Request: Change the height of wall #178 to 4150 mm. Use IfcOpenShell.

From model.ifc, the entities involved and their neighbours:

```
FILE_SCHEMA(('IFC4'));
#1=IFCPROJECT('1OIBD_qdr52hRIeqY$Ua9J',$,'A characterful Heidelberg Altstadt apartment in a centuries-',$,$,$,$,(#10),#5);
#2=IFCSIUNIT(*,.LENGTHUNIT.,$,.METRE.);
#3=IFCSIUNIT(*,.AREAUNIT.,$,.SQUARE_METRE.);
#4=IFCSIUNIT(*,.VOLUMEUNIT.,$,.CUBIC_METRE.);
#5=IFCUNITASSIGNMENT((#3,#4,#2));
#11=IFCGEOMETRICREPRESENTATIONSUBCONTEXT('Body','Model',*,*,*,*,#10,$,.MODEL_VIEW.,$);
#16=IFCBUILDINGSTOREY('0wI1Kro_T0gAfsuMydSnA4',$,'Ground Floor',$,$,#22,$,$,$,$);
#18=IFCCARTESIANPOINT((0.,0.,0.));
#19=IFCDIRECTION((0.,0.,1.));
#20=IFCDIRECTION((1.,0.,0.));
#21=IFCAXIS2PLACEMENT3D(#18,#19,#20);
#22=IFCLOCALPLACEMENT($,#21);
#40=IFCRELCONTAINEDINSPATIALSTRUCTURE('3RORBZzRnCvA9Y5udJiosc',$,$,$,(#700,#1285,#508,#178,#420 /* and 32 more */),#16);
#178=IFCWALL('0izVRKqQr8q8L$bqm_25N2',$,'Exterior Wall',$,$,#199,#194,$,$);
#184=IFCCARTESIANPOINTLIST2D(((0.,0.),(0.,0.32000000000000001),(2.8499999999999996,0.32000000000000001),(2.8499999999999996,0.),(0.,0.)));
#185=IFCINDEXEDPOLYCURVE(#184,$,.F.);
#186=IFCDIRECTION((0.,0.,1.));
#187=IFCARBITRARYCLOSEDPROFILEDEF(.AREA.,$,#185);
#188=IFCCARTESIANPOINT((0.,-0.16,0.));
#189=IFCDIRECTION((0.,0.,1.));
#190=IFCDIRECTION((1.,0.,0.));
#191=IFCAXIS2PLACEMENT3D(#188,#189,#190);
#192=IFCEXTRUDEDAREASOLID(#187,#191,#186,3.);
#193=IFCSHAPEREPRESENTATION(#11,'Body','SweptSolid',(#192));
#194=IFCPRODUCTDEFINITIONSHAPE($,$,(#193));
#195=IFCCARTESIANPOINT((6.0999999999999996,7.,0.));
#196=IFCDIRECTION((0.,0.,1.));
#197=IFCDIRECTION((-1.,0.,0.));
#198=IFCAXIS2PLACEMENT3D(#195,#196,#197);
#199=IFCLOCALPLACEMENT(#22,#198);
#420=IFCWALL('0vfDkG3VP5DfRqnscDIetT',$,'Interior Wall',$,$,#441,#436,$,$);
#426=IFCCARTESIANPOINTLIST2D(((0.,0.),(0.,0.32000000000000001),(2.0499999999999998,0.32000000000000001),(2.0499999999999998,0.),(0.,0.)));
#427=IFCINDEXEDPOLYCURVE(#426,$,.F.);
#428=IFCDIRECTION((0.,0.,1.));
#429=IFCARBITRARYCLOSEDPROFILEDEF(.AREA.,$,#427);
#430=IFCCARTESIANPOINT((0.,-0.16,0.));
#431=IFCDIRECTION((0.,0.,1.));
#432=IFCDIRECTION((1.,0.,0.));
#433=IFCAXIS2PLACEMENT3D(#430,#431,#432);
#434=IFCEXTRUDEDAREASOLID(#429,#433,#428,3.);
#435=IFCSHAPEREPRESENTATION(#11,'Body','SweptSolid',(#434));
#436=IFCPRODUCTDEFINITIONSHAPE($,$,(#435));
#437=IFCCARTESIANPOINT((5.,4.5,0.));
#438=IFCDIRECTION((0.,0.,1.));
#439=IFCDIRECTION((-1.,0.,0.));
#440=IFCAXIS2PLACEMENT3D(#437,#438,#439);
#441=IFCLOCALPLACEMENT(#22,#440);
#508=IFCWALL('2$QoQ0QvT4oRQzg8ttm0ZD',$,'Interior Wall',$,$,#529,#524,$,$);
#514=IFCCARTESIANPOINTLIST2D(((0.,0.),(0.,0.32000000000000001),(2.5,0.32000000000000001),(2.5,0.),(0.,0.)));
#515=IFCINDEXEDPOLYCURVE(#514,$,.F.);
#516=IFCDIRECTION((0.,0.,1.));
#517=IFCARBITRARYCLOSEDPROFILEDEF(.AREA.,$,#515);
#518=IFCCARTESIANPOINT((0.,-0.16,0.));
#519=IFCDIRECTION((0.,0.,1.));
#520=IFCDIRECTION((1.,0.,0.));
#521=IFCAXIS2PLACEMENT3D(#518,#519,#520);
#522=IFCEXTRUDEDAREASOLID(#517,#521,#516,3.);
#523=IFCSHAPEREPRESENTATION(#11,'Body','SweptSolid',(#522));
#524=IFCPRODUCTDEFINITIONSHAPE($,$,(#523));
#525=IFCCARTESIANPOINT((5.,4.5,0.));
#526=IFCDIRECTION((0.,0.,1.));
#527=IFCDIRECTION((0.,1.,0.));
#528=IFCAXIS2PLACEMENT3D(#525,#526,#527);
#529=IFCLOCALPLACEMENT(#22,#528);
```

```python
import ifcopenshell
import ifcopenshell.geom
import ifcopenshell.util.representation
import ifcopenshell.util.shape
import ifcopenshell.util.unit

model = ifcopenshell.open("model.ifc")
unit_scale = ifcopenshell.util.unit.calculate_unit_scale(model)
settings = ifcopenshell.geom.settings()


def volume(element):
    """Net volume in cubic metres, openings subtracted."""
    shape = ifcopenshell.geom.create_shape(settings, element)
    return ifcopenshell.util.shape.get_volume(shape.geometry)


wall = model.by_guid("0izVRKqQr8q8L$bqm_25N2")
before = volume(wall)

body = ifcopenshell.util.representation.get_representation(wall, "Model", "Body")
solid = body.Items[0]
old_height = solid.Depth
solid.Depth = 4.15 / unit_scale
after = volume(wall)

print(f"height {old_height:g} -> {solid.Depth:g}, volume {before:.3f} -> {after:.3f} m3")

model.write("model_edited.ifc")
```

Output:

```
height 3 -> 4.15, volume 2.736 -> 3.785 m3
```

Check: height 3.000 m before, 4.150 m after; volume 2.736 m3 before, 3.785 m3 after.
